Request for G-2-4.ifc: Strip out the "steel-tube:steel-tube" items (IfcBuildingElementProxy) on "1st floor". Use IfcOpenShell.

First a look at what the model holds.

```python
import ifcopenshell
import ifcopenshell.util.element

model = ifcopenshell.open("G-2-4.ifc")
print(model.schema)
storey = next(s for s in model.by_type("IfcBuildingStorey") if s.Name == "1st floor")
proxies = [e for e in ifcopenshell.util.element.get_decomposition(storey) if e.is_a("IfcBuildingElementProxy")]
seen = {}
for e in proxies:
    element_type = ifcopenshell.util.element.get_type(e)
    name = element_type.Name if element_type not in (None, e) else None
    seen[name] = seen.get(name, 0) + 1
for name, count in sorted(seen.items(), key=str):
    print(count, "x", name)
```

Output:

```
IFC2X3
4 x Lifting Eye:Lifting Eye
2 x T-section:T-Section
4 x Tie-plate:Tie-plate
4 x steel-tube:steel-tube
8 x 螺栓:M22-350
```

```python
import ifcopenshell
import ifcopenshell.api.root
import ifcopenshell.util.element

model = ifcopenshell.open("G-2-4.ifc")

storey = next(s for s in model.by_type("IfcBuildingStorey") if s.Name == "1st floor")
proxies = [e for e in ifcopenshell.util.element.get_decomposition(storey) if e.is_a("IfcBuildingElementProxy")]
targets = [e for e in proxies if (t := ifcopenshell.util.element.get_type(e)) not in (None, e) and t.Name == "steel-tube:steel-tube"]

for e in targets:
    ifcopenshell.api.root.remove_product(model, product=e)
print(len(targets), "removed")

model.write("G-2-4_v2.ifc")
```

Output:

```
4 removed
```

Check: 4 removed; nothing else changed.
